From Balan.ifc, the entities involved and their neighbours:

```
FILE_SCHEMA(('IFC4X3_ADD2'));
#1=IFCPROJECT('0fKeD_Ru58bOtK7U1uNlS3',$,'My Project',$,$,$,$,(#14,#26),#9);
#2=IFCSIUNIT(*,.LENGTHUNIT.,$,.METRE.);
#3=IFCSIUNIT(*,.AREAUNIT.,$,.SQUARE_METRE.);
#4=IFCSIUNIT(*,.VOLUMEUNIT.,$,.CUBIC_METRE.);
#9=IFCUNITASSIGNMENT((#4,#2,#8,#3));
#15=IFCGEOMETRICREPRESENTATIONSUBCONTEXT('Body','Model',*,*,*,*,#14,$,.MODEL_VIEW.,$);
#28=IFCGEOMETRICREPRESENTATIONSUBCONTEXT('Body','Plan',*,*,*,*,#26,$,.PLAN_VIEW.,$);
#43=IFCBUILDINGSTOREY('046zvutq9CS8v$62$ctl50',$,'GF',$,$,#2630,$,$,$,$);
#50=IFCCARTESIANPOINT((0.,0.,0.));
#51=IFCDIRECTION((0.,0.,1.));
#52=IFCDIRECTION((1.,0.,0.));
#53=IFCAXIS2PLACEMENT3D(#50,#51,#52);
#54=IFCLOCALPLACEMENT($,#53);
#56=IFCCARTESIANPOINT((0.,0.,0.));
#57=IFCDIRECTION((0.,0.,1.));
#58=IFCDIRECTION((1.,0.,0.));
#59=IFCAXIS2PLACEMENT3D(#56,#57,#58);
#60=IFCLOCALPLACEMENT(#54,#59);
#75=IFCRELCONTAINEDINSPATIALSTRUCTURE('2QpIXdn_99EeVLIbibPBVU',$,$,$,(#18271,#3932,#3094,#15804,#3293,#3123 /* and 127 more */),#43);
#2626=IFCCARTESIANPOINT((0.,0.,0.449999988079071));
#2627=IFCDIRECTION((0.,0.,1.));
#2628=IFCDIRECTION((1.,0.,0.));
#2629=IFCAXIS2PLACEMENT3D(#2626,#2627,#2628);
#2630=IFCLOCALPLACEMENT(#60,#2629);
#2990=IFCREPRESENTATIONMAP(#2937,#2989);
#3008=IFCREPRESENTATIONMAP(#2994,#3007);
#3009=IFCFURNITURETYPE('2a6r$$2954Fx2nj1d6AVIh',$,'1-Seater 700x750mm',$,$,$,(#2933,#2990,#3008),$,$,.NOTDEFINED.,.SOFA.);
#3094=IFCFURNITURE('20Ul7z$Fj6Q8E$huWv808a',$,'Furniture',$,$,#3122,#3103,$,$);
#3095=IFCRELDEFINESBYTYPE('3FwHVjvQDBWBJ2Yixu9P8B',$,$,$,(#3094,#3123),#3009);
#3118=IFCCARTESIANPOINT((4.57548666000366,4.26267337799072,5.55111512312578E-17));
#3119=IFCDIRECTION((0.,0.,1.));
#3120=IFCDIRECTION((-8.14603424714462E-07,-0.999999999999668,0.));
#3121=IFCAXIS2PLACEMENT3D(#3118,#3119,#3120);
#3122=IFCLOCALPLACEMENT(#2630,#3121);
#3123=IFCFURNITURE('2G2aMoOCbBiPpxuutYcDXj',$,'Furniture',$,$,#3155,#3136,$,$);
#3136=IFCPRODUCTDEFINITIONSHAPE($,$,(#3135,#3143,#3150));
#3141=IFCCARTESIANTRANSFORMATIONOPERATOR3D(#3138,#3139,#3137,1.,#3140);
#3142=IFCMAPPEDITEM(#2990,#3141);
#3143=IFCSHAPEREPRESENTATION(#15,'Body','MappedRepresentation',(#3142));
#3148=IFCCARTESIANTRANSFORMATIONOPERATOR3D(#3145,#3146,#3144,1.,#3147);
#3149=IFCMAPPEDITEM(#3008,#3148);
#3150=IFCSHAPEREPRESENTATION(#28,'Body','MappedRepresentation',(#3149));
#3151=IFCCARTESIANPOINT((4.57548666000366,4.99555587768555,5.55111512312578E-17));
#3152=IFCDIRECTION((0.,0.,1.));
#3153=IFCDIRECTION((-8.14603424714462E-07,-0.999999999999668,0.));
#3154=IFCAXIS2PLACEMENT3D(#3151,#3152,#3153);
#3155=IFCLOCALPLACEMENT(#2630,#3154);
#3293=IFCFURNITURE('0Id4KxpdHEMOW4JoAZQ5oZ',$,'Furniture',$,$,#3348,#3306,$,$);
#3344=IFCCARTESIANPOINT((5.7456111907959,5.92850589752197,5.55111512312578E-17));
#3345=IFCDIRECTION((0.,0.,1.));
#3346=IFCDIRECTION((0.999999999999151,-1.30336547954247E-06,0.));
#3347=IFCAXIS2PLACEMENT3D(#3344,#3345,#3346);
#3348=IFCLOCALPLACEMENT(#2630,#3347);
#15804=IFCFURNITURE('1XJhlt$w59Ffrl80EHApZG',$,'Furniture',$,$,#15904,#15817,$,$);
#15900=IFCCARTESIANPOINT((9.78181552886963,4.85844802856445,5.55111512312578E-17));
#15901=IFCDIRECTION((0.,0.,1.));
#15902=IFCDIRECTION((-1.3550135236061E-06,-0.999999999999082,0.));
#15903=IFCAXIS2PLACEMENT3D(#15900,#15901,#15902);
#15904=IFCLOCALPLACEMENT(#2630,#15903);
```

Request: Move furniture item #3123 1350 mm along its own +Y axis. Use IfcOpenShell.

```python
import ifcopenshell
import ifcopenshell.api.geometry
import ifcopenshell.util.placement

model = ifcopenshell.open("Balan.ifc")

item = model.by_guid("2G2aMoOCbBiPpxuutYcDXj")
matrix = ifcopenshell.util.placement.get_local_placement(item.ObjectPlacement)
matrix[:3, 3] += matrix[:3, 1] * 1.35
ifcopenshell.api.geometry.edit_object_placement(model, product=item, matrix=matrix, is_si=False)

print(ifcopenshell.util.placement.get_local_placement(item.ObjectPlacement).round(3) + 0.0)

model.write("Balan_updated.ifc")
```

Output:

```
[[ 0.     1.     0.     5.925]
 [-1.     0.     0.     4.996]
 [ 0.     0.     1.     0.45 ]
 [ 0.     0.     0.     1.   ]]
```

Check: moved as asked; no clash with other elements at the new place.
